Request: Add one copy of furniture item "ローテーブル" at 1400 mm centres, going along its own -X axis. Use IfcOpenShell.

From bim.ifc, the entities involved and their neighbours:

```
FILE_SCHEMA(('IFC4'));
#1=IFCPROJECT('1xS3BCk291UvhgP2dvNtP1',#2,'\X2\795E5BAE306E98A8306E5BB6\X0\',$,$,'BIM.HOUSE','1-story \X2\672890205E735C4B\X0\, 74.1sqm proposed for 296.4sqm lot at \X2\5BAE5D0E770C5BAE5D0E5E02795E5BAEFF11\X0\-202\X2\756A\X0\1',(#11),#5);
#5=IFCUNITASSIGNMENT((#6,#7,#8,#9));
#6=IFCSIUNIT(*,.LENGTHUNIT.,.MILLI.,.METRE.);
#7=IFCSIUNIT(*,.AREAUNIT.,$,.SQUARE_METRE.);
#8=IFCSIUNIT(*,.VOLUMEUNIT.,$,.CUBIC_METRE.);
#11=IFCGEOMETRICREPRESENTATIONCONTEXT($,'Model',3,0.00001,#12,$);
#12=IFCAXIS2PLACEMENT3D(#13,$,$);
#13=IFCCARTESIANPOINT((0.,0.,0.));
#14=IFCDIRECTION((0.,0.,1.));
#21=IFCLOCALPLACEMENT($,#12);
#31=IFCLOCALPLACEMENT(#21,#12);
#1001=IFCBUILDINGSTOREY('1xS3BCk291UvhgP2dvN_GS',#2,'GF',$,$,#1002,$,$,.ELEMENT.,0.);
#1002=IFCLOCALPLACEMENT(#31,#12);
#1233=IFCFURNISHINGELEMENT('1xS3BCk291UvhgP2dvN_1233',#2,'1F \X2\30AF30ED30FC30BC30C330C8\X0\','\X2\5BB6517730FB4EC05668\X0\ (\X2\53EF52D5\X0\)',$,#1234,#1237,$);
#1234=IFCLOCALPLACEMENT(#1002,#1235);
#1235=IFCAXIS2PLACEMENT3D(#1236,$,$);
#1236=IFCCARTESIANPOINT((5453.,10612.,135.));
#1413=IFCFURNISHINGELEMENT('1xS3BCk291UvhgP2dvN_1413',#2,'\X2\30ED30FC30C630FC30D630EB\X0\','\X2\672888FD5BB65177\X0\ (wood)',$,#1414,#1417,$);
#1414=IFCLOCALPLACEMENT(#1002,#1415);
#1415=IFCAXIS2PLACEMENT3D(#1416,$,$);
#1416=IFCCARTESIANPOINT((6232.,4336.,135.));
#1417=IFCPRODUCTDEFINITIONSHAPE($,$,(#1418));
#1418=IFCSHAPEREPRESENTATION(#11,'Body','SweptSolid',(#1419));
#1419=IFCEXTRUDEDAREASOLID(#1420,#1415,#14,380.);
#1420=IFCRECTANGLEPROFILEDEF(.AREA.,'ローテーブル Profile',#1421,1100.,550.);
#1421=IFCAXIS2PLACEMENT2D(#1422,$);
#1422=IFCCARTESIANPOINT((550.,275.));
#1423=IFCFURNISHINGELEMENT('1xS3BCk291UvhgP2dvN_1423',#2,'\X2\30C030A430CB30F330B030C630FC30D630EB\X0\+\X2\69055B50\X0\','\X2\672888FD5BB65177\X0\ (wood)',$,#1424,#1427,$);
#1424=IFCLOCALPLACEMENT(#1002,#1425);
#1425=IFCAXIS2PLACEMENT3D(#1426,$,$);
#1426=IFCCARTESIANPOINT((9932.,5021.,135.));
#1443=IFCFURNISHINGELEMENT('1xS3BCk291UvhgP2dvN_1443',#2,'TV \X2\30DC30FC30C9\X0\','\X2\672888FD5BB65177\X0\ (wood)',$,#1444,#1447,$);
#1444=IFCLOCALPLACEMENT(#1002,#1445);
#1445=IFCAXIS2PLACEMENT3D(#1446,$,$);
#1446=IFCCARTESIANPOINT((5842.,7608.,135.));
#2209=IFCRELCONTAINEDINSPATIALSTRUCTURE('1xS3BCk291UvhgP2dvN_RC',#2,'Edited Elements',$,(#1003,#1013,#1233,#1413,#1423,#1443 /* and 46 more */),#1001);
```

```python
import ifcopenshell
import ifcopenshell.api.geometry
import ifcopenshell.api.root
import ifcopenshell.util.element
import ifcopenshell.util.placement

model = ifcopenshell.open("bim.ifc")


def reuse_history(source, copy):
    """copy_class also copies each property set's owner history, people and application; keep the originals."""
    for rel in copy.IsDefinedBy:
        if rel.is_a("IfcRelDefinesByProperties") and (history := rel.RelatingPropertyDefinition.OwnerHistory):
            rel.RelatingPropertyDefinition.OwnerHistory = source.OwnerHistory
            ifcopenshell.util.element.remove_deep2(model, history)


source = model.by_guid("1xS3BCk291UvhgP2dvN_1413")
base = ifcopenshell.util.placement.get_local_placement(source.ObjectPlacement)
step = -base[:3, 0] * 1400.0

for i in range(1, 2):
    copy = ifcopenshell.api.root.copy_class(model, product=source)
    copy.Representation = ifcopenshell.util.element.copy_deep(
        model, source.Representation, exclude=["IfcGeometricRepresentationContext", "IfcRepresentationMap"]
    )
    reuse_history(source, copy)
    matrix = base.copy()
    matrix[:3, 3] += i * step
    print("added at", matrix[:3, 3].round(3) + 0.0)
    ifcopenshell.api.geometry.edit_object_placement(model, product=copy, matrix=matrix, is_si=False)

model.write("bim_rev.ifc")
```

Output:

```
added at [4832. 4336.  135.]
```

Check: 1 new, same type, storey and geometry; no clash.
